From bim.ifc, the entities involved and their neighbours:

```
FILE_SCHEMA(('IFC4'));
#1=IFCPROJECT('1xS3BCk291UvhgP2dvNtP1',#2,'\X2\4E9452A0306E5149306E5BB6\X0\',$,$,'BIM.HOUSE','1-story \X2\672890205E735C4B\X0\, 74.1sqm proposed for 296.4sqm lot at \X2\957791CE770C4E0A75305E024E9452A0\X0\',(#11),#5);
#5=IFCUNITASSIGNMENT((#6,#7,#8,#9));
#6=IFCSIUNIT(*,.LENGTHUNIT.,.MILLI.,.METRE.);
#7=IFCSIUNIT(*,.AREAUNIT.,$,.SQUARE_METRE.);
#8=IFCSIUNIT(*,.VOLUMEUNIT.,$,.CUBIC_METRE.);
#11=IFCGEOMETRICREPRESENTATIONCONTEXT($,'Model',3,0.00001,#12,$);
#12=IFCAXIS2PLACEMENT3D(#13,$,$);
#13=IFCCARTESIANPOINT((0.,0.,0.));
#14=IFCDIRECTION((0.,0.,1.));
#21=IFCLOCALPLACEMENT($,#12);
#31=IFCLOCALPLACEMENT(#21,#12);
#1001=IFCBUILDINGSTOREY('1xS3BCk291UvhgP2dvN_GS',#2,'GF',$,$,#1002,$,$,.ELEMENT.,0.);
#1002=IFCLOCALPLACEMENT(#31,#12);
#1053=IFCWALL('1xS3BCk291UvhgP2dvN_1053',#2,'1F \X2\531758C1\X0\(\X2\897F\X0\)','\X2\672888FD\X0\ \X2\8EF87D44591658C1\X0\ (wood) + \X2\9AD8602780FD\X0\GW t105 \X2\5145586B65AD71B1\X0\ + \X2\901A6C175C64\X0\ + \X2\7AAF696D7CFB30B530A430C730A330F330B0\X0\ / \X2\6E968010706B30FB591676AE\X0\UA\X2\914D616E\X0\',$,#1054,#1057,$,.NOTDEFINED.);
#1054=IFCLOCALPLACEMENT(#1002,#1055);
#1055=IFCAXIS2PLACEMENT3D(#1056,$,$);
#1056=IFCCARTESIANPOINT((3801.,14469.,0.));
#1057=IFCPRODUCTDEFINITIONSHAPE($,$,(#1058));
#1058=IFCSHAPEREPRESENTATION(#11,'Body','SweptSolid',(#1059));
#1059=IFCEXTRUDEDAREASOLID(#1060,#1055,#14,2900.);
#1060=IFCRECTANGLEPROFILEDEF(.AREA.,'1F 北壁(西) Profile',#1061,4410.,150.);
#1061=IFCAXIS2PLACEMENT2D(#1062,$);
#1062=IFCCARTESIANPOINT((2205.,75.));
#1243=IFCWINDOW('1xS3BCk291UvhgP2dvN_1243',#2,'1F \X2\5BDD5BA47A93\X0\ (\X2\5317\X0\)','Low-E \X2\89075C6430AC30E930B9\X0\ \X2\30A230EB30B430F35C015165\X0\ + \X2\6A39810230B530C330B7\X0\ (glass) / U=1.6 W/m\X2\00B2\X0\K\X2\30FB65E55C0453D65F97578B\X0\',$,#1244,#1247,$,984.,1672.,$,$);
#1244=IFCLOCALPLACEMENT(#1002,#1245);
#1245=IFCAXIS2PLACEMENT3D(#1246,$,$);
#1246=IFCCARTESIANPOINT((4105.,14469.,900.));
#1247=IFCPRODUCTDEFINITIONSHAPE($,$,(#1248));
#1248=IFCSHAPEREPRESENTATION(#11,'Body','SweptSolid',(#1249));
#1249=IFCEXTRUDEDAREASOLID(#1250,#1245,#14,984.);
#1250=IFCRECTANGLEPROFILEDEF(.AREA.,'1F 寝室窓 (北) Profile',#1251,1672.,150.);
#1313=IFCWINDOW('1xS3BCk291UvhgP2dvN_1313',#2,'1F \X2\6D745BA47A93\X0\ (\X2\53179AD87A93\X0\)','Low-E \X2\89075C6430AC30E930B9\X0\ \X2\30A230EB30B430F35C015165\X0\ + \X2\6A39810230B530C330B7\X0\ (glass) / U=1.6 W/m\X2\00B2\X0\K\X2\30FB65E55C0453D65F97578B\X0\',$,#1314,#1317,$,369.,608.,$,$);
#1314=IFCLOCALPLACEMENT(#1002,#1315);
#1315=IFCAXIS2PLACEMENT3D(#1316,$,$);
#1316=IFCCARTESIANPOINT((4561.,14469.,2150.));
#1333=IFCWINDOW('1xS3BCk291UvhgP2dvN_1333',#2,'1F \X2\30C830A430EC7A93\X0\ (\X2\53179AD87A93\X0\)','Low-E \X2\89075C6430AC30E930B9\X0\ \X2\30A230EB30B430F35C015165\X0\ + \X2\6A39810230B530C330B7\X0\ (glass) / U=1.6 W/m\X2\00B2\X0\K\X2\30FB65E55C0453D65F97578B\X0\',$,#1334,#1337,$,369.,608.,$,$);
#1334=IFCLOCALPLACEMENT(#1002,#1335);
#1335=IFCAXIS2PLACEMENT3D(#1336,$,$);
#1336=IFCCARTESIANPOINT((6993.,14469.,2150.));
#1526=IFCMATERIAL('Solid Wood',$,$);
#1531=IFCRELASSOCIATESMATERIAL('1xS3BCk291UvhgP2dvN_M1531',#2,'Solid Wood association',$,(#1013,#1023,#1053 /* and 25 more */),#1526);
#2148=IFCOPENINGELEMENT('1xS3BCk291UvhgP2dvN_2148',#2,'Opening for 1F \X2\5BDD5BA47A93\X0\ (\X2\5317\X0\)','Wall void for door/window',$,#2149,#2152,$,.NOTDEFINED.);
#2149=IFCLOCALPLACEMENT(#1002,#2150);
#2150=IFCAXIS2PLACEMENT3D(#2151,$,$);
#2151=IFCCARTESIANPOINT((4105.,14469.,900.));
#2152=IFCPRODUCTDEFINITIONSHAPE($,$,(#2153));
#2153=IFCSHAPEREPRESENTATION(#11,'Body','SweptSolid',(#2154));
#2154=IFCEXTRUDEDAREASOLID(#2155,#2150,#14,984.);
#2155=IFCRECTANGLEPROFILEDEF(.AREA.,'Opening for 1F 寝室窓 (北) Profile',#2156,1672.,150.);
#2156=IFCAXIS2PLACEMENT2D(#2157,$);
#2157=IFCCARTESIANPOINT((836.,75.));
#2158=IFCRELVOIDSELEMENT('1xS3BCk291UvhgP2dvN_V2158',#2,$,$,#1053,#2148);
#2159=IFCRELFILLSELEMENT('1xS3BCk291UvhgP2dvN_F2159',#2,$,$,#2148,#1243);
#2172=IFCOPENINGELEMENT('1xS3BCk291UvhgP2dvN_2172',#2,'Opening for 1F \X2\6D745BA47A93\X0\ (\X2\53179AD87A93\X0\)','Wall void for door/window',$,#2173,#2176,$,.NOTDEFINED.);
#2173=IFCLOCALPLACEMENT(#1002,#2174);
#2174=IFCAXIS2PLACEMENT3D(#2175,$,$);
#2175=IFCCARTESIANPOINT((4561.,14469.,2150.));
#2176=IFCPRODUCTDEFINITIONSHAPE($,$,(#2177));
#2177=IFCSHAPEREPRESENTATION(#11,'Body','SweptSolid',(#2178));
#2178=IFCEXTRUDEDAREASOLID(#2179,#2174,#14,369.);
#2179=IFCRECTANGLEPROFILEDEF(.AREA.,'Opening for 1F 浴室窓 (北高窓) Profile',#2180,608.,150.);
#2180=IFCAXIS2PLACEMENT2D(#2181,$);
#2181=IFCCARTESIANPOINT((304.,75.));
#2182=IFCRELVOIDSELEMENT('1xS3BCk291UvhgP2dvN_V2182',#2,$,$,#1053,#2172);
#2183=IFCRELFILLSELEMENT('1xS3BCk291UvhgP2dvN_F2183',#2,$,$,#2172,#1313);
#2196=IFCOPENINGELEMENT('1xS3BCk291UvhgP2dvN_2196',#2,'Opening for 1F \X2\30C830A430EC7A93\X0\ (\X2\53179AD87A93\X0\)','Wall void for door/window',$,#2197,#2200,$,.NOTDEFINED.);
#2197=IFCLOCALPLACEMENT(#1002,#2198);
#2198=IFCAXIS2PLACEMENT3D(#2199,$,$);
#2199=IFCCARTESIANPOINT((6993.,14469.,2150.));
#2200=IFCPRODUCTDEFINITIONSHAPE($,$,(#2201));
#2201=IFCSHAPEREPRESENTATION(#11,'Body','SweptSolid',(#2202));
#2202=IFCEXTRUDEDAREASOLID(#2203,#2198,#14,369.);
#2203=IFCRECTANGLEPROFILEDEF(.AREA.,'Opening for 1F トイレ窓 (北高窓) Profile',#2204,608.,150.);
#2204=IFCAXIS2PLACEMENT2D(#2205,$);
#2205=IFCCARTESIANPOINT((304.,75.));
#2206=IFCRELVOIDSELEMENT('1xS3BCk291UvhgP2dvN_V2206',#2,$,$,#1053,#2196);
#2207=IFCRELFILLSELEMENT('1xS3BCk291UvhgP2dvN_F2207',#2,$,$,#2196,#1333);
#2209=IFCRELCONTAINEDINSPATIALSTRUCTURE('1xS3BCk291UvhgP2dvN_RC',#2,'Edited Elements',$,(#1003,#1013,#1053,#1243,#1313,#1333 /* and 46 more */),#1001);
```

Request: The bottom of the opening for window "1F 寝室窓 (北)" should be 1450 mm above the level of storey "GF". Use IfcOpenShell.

```python
import numpy as np
import ifcopenshell
import ifcopenshell.api.geometry
import ifcopenshell.geom
import ifcopenshell.util.element
import ifcopenshell.util.placement
import ifcopenshell.util.shape
import ifcopenshell.util.unit

model = ifcopenshell.open("bim.ifc")
unit_scale = ifcopenshell.util.unit.calculate_unit_scale(model)

window = model.by_guid("1xS3BCk291UvhgP2dvN_1243")
opening = window.FillsVoids[0].RelatingOpeningElement
storey = ifcopenshell.util.element.get_container(window, ifc_class="IfcBuildingStorey")
level = ifcopenshell.util.placement.get_local_placement(storey.ObjectPlacement)[2, 3]

# The opening's origin need not be at the sill, so measure its lowest point.
shape = ifcopenshell.geom.create_shape(ifcopenshell.geom.settings(), opening)
bottom = ifcopenshell.util.shape.get_shape_bottom_elevation(shape, shape.geometry) / unit_scale
dz = level + 1450.0 - bottom

shift = np.array([0.0, 0.0, dz])
# The window is not placed relative to its opening, so move both.
for product in (opening, window):
    matrix = ifcopenshell.util.placement.get_local_placement(product.ObjectPlacement)
    matrix[:3, 3] += shift
    ifcopenshell.api.geometry.edit_object_placement(model, product=product, matrix=matrix, is_si=False)

print(f"moved by {dz * unit_scale:+.3f} m")

model.write("bim_rev.ifc")
```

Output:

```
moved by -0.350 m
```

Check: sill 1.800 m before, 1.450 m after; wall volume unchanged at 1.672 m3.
